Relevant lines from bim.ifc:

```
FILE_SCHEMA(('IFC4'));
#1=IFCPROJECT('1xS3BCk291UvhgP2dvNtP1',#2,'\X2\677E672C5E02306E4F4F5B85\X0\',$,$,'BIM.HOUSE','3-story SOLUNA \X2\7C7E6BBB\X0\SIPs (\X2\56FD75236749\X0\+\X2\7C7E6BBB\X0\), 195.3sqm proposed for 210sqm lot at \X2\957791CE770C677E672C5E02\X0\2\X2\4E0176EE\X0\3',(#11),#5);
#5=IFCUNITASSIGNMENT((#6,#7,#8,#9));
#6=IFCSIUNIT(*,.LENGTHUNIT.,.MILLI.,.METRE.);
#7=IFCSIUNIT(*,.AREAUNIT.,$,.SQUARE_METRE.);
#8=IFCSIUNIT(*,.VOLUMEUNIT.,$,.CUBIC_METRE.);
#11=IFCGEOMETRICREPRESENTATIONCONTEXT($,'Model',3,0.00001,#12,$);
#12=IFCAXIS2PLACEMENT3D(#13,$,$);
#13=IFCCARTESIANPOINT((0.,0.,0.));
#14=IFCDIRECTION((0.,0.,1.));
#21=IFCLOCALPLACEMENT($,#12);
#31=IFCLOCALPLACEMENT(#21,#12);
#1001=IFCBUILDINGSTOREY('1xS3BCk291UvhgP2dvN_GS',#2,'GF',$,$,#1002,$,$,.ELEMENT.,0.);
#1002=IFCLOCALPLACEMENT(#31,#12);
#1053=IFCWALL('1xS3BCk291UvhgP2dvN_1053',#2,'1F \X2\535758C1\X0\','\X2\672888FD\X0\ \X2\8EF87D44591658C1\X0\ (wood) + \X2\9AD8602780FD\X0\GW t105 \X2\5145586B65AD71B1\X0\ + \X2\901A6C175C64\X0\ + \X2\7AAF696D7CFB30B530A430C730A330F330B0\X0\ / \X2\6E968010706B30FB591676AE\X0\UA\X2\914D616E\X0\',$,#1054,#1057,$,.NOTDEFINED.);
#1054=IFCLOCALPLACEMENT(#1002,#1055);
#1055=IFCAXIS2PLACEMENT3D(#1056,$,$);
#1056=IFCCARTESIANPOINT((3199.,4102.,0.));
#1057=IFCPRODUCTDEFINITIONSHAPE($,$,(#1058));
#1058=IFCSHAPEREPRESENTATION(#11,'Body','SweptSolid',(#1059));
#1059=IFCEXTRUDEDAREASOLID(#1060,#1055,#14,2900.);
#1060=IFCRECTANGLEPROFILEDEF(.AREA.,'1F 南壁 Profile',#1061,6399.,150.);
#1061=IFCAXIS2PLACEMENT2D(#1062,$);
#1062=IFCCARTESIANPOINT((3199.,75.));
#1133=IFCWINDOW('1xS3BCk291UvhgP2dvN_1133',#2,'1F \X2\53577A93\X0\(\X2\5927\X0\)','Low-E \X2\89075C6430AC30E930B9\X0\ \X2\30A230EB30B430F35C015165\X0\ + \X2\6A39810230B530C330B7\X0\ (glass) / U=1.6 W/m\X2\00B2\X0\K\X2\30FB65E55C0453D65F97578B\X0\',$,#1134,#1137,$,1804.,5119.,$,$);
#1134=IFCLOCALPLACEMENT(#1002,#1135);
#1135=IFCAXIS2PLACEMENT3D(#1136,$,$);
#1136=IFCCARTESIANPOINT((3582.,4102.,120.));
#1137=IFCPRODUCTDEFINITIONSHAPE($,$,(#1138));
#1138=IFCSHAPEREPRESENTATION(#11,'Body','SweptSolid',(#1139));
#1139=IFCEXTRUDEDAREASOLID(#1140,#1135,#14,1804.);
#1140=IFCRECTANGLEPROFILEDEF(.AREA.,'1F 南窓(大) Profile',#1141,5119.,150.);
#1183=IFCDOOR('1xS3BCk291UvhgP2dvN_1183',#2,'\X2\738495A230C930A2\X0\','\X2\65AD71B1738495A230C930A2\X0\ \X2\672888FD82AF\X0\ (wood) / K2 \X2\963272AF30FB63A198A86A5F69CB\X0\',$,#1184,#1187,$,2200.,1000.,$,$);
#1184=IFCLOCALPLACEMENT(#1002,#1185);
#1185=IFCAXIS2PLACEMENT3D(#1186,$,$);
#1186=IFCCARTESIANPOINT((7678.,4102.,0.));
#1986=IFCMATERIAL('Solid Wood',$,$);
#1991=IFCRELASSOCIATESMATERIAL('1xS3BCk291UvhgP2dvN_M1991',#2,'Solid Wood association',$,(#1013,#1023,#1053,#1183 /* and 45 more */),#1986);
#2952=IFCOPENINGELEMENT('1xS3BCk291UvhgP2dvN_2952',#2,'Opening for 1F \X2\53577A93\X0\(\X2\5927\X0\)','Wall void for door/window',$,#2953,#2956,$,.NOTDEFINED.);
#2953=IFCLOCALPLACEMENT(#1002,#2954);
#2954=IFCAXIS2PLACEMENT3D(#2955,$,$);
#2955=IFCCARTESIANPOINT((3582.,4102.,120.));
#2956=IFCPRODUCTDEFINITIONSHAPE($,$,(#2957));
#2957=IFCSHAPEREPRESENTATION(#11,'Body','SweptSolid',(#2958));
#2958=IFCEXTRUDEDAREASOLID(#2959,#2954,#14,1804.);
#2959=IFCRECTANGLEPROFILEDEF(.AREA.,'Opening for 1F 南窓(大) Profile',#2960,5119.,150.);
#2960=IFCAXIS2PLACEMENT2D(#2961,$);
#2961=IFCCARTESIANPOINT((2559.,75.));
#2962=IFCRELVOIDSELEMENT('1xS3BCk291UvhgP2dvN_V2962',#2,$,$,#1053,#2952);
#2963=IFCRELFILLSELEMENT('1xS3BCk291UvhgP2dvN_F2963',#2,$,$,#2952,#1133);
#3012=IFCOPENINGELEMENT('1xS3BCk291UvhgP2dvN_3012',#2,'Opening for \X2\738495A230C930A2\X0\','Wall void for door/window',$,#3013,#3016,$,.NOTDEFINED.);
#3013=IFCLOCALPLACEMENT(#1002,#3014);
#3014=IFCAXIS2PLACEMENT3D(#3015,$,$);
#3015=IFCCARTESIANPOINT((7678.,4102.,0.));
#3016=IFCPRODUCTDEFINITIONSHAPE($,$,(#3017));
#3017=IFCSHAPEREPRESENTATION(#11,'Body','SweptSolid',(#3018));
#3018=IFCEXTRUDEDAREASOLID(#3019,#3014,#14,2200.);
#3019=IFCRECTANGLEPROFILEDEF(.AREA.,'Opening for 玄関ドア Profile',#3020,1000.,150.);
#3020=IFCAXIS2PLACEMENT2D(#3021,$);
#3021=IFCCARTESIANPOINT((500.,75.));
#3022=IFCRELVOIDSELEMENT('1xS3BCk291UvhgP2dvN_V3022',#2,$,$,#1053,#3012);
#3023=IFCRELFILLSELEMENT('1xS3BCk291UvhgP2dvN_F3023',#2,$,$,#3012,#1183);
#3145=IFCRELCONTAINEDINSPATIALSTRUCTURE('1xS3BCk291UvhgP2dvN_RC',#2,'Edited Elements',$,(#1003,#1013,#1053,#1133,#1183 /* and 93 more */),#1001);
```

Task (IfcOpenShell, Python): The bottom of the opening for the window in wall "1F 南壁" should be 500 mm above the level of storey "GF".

```python
import numpy as np
import ifcopenshell
import ifcopenshell.api.geometry
import ifcopenshell.geom
import ifcopenshell.util.element
import ifcopenshell.util.placement
import ifcopenshell.util.shape
import ifcopenshell.util.unit

model = ifcopenshell.open("bim.ifc")
unit_scale = ifcopenshell.util.unit.calculate_unit_scale(model)

window = model.by_guid("1xS3BCk291UvhgP2dvN_1133")
opening = window.FillsVoids[0].RelatingOpeningElement
storey = ifcopenshell.util.element.get_container(window, ifc_class="IfcBuildingStorey")
level = ifcopenshell.util.placement.get_local_placement(storey.ObjectPlacement)[2, 3]

# The opening's origin need not be at the sill, so measure its lowest point.
shape = ifcopenshell.geom.create_shape(ifcopenshell.geom.settings(), opening)
bottom = ifcopenshell.util.shape.get_shape_bottom_elevation(shape, shape.geometry) / unit_scale
dz = level + 500.0 - bottom

shift = np.array([0.0, 0.0, dz])
# The window is not placed relative to its opening, so move both.
for product in (opening, window):
    matrix = ifcopenshell.util.placement.get_local_placement(product.ObjectPlacement)
    matrix[:3, 3] += shift
    ifcopenshell.api.geometry.edit_object_placement(model, product=product, matrix=matrix, is_si=False)

print(f"moved by {dz * unit_scale:+.3f} m")

model.write("bim-out.ifc")
```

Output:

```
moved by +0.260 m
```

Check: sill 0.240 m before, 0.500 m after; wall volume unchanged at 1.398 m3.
